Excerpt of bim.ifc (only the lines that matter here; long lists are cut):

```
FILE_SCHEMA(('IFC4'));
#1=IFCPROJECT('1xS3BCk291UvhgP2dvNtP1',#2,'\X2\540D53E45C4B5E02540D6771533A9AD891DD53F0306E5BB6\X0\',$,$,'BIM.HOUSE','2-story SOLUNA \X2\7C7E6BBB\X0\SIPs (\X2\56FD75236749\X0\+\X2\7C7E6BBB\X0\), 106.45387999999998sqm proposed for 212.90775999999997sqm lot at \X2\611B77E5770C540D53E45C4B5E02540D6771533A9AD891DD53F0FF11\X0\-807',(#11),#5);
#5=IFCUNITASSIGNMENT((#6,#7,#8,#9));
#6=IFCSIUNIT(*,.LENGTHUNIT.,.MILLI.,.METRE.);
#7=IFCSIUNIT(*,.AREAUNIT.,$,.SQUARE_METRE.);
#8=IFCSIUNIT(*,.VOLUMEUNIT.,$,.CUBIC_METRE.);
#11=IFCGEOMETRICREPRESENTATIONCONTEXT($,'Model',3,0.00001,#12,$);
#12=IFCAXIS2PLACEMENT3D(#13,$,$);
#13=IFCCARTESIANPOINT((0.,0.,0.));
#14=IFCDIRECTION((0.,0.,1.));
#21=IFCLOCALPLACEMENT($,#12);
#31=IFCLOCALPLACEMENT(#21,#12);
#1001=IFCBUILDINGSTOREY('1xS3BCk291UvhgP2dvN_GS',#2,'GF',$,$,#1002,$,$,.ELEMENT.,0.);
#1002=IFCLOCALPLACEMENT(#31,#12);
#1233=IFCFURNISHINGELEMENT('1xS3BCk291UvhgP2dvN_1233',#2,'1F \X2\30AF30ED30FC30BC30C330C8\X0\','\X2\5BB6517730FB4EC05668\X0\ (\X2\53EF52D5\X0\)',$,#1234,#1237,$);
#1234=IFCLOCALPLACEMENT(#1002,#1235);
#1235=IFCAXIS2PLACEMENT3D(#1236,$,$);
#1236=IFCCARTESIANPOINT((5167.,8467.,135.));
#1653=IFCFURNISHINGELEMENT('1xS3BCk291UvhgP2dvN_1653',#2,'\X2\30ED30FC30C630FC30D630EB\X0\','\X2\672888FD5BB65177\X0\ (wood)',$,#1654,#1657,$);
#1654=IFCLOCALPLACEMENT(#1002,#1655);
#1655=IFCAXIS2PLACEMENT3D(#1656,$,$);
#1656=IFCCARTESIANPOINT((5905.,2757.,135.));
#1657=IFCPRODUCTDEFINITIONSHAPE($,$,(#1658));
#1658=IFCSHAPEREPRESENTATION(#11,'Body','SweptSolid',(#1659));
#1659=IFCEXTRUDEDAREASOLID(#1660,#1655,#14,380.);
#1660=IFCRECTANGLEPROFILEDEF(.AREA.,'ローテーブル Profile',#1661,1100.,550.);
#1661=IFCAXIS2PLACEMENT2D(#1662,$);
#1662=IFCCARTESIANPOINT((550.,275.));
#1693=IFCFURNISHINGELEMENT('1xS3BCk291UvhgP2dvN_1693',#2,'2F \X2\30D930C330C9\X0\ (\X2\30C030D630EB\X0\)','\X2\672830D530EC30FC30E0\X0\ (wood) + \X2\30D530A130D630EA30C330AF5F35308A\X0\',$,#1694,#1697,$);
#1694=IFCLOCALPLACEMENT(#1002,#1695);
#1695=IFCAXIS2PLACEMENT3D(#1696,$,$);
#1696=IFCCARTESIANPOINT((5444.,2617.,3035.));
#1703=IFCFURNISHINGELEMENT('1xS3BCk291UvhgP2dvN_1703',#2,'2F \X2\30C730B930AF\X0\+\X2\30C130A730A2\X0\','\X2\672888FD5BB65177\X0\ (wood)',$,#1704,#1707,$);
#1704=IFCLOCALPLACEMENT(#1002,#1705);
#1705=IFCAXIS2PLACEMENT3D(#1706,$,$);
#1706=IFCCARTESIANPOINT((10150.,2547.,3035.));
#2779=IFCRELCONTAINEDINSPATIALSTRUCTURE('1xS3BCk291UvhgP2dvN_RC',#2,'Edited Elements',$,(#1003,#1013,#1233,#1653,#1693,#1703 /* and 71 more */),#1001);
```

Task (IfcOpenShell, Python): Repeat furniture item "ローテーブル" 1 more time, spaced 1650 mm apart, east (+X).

```python
import numpy as np
import ifcopenshell
import ifcopenshell.api.geometry
import ifcopenshell.api.root
import ifcopenshell.util.element
import ifcopenshell.util.placement

model = ifcopenshell.open("bim.ifc")


def reuse_history(source, copy):
    """copy_class also copies each property set's owner history, people and application; keep the originals."""
    for rel in copy.IsDefinedBy:
        if rel.is_a("IfcRelDefinesByProperties") and (history := rel.RelatingPropertyDefinition.OwnerHistory):
            rel.RelatingPropertyDefinition.OwnerHistory = source.OwnerHistory
            ifcopenshell.util.element.remove_deep2(model, history)


source = model.by_guid("1xS3BCk291UvhgP2dvN_1653")
base = ifcopenshell.util.placement.get_local_placement(source.ObjectPlacement)
step = np.array([1.0, 0.0, 0.0]) * 1650.0

for i in range(1, 2):
    copy = ifcopenshell.api.root.copy_class(model, product=source)
    copy.Representation = ifcopenshell.util.element.copy_deep(
        model, source.Representation, exclude=["IfcGeometricRepresentationContext", "IfcRepresentationMap"]
    )
    reuse_history(source, copy)
    matrix = base.copy()
    matrix[:3, 3] += i * step
    print("added at", matrix[:3, 3].round(3) + 0.0)
    ifcopenshell.api.geometry.edit_object_placement(model, product=copy, matrix=matrix, is_si=False)

model.write("bim_edited.ifc")
```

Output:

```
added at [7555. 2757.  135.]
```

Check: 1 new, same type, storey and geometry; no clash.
